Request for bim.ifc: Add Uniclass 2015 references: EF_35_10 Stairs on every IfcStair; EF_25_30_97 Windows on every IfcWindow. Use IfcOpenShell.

First a look at what the model holds.

```python
import ifcopenshell

model = ifcopenshell.open("bim.ifc")
print(model.schema)
print("classifications:", [c.Name for c in model.by_type("IfcClassification")])
for ifc_class in ("IfcDoor", "IfcRoof", "IfcStair", "IfcWall", "IfcWindow"):
    print(ifc_class, len(model.by_type(ifc_class)))
```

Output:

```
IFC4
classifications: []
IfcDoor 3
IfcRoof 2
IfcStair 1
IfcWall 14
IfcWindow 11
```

```python
import ifcopenshell
import ifcopenshell.api.classification

model = ifcopenshell.open("bim.ifc")

system = ifcopenshell.api.classification.add_classification(model, classification="Uniclass 2015")

codes = {
    "IfcStair": ("EF_35_10", "Stairs"),
    "IfcWindow": ("EF_25_30_97", "Windows"),
}
for ifc_class, (code, name) in codes.items():
    products = model.by_type(ifc_class)
    ifcopenshell.api.classification.add_reference(
        model, products=products, classification=system, identification=code, name=name
    )
    print(code, len(products))

model.write("bim-out.ifc")
```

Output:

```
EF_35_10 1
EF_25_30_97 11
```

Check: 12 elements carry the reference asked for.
